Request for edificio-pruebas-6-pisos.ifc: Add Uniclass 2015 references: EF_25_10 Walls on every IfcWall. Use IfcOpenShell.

First a look at what the model holds.

```python
import ifcopenshell

model = ifcopenshell.open("edificio-pruebas-6-pisos.ifc")
print(model.schema)
print("classifications:", [c.Name for c in model.by_type("IfcClassification")])
for ifc_class in ("IfcDoor", "IfcRoof", "IfcStair", "IfcWall", "IfcWindow"):
    print(ifc_class, len(model.by_type(ifc_class)))
```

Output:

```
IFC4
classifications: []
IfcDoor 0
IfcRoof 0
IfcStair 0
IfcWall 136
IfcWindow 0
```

```python
import ifcopenshell
import ifcopenshell.api.classification

model = ifcopenshell.open("edificio-pruebas-6-pisos.ifc")

system = ifcopenshell.api.classification.add_classification(model, classification="Uniclass 2015")

codes = {
    "IfcWall": ("EF_25_10", "Walls"),
}
for ifc_class, (code, name) in codes.items():
    products = model.by_type(ifc_class)
    ifcopenshell.api.classification.add_reference(
        model, products=products, classification=system, identification=code, name=name
    )
    print(code, len(products))

model.write("edificio-pruebas-6-pisos_rev.ifc")
```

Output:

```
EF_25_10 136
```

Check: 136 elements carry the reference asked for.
